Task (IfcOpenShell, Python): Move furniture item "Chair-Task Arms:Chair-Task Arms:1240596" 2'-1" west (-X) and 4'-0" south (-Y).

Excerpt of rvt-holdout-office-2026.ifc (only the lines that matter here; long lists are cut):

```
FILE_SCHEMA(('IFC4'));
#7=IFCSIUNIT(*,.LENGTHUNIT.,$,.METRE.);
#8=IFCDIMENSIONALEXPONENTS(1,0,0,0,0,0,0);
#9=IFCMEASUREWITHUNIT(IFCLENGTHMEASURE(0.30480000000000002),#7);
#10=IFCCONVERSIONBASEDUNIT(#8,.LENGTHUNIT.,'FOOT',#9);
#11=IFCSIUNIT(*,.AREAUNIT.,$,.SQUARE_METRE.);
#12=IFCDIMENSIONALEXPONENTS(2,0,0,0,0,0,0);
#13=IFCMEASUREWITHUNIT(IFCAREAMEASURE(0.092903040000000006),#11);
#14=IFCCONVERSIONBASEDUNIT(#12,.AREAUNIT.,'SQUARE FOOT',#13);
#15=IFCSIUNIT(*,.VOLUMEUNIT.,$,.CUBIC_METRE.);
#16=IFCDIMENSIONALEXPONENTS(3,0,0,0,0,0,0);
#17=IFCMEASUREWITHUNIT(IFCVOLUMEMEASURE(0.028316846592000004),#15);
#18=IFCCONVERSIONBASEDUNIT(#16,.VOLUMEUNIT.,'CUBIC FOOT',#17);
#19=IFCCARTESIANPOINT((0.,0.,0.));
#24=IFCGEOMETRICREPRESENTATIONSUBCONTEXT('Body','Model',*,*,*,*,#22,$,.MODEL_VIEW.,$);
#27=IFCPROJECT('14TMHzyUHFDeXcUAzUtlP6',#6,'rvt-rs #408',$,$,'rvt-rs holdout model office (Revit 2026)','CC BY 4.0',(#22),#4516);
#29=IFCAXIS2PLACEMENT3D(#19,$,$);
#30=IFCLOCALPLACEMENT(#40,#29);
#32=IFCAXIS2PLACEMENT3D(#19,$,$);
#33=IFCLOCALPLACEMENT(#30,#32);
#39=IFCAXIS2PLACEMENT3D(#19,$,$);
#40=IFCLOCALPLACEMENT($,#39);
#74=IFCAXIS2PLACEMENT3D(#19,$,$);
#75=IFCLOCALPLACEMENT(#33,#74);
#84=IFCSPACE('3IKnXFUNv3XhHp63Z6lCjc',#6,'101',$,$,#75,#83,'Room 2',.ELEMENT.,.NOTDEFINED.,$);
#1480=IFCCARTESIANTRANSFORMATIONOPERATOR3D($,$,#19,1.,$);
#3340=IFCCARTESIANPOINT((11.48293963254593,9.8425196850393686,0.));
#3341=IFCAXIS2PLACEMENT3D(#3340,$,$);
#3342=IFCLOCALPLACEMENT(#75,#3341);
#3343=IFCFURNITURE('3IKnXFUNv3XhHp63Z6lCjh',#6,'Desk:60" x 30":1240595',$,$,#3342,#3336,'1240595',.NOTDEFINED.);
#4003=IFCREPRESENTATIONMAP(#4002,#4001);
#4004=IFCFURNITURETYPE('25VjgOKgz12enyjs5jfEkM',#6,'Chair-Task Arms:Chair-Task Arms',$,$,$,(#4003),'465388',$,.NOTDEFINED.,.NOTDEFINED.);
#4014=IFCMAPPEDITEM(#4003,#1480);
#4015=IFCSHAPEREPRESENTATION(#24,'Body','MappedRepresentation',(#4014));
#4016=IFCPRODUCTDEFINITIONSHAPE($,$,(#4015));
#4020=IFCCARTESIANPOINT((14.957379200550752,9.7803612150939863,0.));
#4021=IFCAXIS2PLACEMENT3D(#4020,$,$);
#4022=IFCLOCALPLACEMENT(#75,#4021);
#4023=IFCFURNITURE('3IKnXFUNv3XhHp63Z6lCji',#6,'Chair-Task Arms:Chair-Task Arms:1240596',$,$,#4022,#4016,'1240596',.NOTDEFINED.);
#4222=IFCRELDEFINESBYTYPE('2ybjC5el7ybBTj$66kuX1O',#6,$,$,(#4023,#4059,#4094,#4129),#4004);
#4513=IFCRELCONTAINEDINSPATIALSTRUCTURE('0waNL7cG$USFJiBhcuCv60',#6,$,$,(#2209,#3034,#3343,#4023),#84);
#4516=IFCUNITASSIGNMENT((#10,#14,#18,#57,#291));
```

```python
import ifcopenshell
import ifcopenshell.api.geometry
import ifcopenshell.util.placement
import ifcopenshell.util.unit

model = ifcopenshell.open("rvt-holdout-office-2026.ifc")
unit_scale = ifcopenshell.util.unit.calculate_unit_scale(model)

item = model.by_guid("3IKnXFUNv3XhHp63Z6lCji")
matrix = ifcopenshell.util.placement.get_local_placement(item.ObjectPlacement)
matrix[0, 3] -= 25 * 0.0254 / unit_scale
matrix[1, 3] -= 48 * 0.0254 / unit_scale
ifcopenshell.api.geometry.edit_object_placement(model, product=item, matrix=matrix, is_si=False)

print(ifcopenshell.util.placement.get_local_placement(item.ObjectPlacement).round(3) + 0.0)

model.write("rvt-holdout-office-2026_rev.ifc")
```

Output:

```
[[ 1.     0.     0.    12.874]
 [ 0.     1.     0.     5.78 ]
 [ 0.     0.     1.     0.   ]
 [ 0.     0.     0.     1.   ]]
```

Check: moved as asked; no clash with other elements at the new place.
